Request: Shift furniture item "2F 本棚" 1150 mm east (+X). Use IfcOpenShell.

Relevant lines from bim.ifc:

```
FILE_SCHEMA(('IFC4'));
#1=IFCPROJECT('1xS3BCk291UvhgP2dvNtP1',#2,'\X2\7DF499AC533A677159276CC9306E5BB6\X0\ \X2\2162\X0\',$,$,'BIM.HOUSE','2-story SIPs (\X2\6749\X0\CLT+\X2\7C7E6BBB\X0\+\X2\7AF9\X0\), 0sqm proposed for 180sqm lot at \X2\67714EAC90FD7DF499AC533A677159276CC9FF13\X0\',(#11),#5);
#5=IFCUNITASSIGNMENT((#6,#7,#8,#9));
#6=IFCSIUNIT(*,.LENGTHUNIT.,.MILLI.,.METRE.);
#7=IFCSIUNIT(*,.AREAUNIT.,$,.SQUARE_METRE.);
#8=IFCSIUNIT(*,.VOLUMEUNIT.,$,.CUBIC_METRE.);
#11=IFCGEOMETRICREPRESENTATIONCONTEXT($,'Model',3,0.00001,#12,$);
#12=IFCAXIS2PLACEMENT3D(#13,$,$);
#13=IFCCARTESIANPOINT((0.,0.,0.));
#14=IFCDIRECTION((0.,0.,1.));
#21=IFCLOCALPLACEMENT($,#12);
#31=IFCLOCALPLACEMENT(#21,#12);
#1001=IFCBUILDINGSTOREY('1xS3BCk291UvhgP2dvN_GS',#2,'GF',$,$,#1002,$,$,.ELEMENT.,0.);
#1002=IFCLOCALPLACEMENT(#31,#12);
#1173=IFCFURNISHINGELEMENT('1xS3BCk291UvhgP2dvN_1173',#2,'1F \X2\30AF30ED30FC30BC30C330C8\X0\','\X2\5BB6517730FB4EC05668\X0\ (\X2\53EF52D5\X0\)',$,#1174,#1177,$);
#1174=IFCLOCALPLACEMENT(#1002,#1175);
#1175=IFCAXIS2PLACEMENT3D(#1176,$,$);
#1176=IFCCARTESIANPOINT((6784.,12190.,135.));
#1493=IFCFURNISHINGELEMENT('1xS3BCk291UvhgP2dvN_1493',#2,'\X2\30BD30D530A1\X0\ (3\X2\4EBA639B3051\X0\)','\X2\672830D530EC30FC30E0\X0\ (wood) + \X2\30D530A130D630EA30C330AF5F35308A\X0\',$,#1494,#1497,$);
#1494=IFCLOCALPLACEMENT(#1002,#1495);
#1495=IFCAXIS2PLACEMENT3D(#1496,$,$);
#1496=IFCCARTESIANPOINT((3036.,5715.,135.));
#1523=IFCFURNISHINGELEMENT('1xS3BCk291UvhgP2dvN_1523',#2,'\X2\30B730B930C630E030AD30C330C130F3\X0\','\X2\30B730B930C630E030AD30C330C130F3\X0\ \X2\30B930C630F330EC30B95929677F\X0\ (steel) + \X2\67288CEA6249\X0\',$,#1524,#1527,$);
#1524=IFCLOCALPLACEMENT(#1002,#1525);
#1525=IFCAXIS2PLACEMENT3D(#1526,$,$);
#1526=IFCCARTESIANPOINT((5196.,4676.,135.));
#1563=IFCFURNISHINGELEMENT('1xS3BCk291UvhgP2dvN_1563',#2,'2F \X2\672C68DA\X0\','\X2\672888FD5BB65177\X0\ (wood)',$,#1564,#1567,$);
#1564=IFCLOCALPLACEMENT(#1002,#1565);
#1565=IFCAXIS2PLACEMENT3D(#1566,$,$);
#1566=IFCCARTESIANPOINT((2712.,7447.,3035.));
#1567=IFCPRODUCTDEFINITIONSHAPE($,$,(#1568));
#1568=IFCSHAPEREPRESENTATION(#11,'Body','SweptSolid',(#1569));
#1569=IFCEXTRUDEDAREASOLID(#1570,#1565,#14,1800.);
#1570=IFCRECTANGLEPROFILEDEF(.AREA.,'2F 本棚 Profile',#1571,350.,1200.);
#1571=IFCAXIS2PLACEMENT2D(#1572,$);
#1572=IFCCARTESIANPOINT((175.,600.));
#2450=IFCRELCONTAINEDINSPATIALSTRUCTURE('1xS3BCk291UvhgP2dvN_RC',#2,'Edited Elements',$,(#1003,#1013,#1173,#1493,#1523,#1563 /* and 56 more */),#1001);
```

```python
import ifcopenshell
import ifcopenshell.api.geometry
import ifcopenshell.util.placement
import ifcopenshell.util.unit

model = ifcopenshell.open("bim.ifc")
unit_scale = ifcopenshell.util.unit.calculate_unit_scale(model)

item = model.by_id(1563)
matrix = ifcopenshell.util.placement.get_local_placement(item.ObjectPlacement)
matrix[0, 3] += 1.15 / unit_scale
ifcopenshell.api.geometry.edit_object_placement(model, product=item, matrix=matrix, is_si=False)

print(ifcopenshell.util.placement.get_local_placement(item.ObjectPlacement).round(3) + 0.0)

model.write("bim-out.ifc")
```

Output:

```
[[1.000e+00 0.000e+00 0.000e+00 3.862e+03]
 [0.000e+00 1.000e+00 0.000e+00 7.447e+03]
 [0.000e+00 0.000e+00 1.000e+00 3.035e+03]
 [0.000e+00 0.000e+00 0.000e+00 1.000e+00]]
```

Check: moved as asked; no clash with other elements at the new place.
